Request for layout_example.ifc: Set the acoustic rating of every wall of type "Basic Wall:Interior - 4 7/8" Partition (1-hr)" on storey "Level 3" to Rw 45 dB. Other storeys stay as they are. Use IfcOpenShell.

First a look at what the model holds.

```python
import ifcopenshell
import ifcopenshell.util.element

model = ifcopenshell.open("layout_example.ifc")
print(model.schema)
storey = next(s for s in model.by_type("IfcBuildingStorey") if s.Name == "Level 3")
walls = [e for e in ifcopenshell.util.element.get_decomposition(storey) if e.is_a("IfcWall")]
seen = {}
for e in walls:
    element_type = ifcopenshell.util.element.get_type(e)
    key = (element_type.Name if element_type != e and element_type else None, ifcopenshell.util.element.get_pset(e, "Pset_WallCommon", "AcousticRating"))
    seen[key] = seen.get(key, 0) + 1
for (name, value), count in sorted(seen.items(), key=str):
    print(count, "x", name, "|", value)
```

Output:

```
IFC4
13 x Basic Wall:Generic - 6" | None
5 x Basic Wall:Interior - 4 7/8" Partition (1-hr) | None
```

```python
import ifcopenshell
import ifcopenshell.api.pset
import ifcopenshell.util.element

model = ifcopenshell.open("layout_example.ifc")

storey = next(s for s in model.by_type("IfcBuildingStorey") if s.Name == "Level 3")
walls = [e for e in ifcopenshell.util.element.get_decomposition(storey) if e.is_a("IfcWall")]

count = 0
for e in walls:
    element_type = ifcopenshell.util.element.get_type(e)
    if element_type in (None, e) or element_type.Name != 'Basic Wall:Interior - 4 7/8" Partition (1-hr)':
        continue
    # add_pset returns the element's existing set when there is one.
    pset = ifcopenshell.api.pset.add_pset(model, product=e, name="Pset_WallCommon")
    ifcopenshell.api.pset.edit_pset(model, pset=pset, properties={"AcousticRating": "Rw 45 dB"})
    count += 1

print(count, "walls updated")

model.write("layout_example_v2.ifc")
```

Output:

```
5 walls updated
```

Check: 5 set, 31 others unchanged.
